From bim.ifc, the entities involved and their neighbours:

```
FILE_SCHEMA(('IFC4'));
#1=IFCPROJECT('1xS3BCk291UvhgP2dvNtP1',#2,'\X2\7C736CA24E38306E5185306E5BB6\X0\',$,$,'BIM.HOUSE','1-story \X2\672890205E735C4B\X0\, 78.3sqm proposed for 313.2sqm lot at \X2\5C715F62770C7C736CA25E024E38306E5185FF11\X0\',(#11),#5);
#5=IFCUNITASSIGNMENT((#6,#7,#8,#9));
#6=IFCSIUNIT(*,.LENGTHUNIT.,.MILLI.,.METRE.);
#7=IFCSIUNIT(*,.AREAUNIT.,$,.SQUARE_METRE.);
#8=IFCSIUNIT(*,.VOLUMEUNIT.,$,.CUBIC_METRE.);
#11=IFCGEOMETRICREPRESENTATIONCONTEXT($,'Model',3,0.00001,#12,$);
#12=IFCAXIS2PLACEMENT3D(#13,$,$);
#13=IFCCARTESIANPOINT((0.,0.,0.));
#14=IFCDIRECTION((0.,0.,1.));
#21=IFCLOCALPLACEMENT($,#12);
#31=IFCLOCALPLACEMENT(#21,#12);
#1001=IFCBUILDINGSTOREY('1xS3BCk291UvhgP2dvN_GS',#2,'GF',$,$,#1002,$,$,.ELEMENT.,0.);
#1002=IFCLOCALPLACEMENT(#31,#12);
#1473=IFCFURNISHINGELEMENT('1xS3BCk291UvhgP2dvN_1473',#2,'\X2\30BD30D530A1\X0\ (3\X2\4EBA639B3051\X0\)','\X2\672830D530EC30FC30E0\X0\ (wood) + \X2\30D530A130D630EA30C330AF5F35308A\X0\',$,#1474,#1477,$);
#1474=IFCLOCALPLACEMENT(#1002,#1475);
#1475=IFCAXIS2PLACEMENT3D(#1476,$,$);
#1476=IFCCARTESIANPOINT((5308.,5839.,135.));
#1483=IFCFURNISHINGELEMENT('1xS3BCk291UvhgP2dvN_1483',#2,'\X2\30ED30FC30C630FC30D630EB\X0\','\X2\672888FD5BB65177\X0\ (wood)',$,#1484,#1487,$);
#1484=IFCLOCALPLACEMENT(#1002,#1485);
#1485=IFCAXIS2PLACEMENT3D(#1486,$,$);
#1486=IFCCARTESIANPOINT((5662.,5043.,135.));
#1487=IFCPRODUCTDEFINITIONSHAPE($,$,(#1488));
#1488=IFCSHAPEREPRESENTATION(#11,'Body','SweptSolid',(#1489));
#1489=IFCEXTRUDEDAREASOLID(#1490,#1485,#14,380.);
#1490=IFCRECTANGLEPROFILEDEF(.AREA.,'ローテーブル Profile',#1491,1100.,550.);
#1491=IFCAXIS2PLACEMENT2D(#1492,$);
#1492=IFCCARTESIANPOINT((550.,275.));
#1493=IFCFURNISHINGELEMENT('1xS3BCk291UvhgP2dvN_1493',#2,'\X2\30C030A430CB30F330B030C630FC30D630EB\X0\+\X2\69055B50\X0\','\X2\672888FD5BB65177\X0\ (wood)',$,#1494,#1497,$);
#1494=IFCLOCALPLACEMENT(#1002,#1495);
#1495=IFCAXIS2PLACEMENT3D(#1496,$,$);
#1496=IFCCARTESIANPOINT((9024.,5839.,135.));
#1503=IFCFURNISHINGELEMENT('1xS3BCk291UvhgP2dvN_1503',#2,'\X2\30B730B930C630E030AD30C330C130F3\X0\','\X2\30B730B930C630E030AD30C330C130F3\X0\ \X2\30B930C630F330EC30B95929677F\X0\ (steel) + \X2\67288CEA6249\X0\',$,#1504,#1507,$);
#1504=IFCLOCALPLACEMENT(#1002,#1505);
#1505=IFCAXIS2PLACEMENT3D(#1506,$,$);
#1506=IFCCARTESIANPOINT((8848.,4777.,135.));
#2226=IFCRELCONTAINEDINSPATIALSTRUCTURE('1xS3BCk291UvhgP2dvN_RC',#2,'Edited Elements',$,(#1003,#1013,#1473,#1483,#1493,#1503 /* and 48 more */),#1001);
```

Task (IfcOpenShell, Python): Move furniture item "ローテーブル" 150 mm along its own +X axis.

```python
import ifcopenshell
import ifcopenshell.api.geometry
import ifcopenshell.util.placement

model = ifcopenshell.open("bim.ifc")

item = model.by_guid("1xS3BCk291UvhgP2dvN_1483")
matrix = ifcopenshell.util.placement.get_local_placement(item.ObjectPlacement)
matrix[:3, 3] += matrix[:3, 0] * 150.0
ifcopenshell.api.geometry.edit_object_placement(model, product=item, matrix=matrix, is_si=False)

print(ifcopenshell.util.placement.get_local_placement(item.ObjectPlacement).round(3) + 0.0)

model.write("bim_v2.ifc")
```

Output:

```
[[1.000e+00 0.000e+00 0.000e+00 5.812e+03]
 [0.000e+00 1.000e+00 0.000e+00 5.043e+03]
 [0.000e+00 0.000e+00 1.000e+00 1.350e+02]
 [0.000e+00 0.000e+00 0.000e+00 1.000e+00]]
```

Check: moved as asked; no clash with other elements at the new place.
